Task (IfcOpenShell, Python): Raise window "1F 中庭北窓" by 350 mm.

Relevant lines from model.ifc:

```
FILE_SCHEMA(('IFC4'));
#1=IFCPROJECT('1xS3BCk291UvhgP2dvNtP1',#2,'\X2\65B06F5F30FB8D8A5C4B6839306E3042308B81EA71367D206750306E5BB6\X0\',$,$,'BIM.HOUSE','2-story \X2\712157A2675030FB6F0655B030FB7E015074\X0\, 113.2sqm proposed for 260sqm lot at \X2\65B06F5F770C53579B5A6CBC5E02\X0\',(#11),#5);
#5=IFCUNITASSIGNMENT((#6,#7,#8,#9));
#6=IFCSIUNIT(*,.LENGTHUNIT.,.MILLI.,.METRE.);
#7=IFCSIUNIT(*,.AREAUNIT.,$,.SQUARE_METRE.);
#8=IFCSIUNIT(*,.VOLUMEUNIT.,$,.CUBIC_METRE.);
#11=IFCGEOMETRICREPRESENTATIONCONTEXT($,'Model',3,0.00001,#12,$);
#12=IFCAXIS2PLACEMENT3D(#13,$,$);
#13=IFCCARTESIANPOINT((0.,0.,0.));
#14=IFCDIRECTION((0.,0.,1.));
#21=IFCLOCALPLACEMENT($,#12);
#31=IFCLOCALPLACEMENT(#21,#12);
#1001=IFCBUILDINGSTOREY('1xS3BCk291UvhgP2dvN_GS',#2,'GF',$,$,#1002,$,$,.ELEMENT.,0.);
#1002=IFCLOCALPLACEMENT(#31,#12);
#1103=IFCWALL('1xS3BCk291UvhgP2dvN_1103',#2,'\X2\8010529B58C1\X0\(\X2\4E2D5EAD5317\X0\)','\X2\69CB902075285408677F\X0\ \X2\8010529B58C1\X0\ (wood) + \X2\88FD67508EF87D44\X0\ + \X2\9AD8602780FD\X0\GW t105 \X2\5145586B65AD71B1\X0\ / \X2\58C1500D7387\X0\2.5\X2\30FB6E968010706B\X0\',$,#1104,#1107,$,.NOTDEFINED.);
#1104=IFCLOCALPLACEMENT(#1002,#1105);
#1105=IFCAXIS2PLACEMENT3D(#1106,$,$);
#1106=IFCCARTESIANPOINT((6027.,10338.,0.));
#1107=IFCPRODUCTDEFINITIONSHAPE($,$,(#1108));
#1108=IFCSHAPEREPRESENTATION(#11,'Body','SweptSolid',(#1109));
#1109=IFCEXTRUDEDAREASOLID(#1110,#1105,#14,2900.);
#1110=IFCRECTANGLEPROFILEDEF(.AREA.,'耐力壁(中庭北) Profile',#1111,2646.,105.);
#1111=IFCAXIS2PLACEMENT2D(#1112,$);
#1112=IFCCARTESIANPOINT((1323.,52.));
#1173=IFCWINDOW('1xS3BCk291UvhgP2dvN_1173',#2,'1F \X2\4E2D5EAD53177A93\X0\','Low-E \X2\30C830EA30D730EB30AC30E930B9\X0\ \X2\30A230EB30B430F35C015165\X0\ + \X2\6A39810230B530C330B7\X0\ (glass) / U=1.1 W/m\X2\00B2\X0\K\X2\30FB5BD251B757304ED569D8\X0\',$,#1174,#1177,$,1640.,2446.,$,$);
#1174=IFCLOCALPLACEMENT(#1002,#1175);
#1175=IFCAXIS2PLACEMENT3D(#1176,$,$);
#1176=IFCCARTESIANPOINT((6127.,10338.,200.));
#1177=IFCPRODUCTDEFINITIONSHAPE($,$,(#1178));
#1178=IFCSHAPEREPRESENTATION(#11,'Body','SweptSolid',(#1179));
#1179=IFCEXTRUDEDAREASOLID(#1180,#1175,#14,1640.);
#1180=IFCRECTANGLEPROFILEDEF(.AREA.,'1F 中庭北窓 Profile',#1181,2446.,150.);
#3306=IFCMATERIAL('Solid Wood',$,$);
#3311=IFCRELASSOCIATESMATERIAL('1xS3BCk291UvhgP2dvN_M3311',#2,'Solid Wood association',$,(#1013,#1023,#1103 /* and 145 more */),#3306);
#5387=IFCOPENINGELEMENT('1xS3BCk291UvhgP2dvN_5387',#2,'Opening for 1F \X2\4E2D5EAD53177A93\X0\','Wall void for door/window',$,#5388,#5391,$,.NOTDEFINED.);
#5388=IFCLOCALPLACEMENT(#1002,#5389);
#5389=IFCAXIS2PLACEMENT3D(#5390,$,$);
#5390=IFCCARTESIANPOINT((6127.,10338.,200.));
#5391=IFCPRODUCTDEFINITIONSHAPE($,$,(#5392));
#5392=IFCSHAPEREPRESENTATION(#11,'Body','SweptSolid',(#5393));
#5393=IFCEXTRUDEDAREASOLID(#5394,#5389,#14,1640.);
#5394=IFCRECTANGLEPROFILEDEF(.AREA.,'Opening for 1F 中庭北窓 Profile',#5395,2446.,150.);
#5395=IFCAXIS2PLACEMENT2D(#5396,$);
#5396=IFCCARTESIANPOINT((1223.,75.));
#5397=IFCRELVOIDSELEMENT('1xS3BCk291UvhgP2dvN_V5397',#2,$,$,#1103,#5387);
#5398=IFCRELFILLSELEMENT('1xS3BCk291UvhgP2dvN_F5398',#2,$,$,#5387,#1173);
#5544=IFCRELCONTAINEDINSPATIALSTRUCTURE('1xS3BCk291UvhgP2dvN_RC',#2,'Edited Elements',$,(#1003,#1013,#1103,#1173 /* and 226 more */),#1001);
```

```python
import numpy as np
import ifcopenshell
import ifcopenshell.api.geometry
import ifcopenshell.util.placement
import ifcopenshell.util.unit

model = ifcopenshell.open("model.ifc")
unit_scale = ifcopenshell.util.unit.calculate_unit_scale(model)

window = model.by_id(1173)
opening = window.FillsVoids[0].RelatingOpeningElement
dz = 350.0

shift = np.array([0.0, 0.0, dz])
# The window is not placed relative to its opening, so move both.
for product in (opening, window):
    matrix = ifcopenshell.util.placement.get_local_placement(product.ObjectPlacement)
    matrix[:3, 3] += shift
    ifcopenshell.api.geometry.edit_object_placement(model, product=product, matrix=matrix, is_si=False)

print(f"moved by {dz * unit_scale:+.3f} m")

model.write("model_updated.ifc")
```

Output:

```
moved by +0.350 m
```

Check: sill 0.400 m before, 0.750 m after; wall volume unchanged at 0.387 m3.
